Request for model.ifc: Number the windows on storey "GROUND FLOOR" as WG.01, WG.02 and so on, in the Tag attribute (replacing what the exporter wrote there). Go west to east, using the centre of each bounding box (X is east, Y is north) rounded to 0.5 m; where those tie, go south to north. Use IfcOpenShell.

First a look at what the model holds.

```python
import ifcopenshell
import ifcopenshell.util.element
import ifcopenshell.util.placement

model = ifcopenshell.open("model.ifc")
print(model.schema)
storey = next(s for s in model.by_type("IfcBuildingStorey") if s.Name == "GROUND FLOOR")
windows = [e for e in ifcopenshell.util.element.get_decomposition(storey) if e.is_a("IfcWindow")]
for e in sorted(windows, key=lambda e: e.id()):
    origin = ifcopenshell.util.placement.get_local_placement(e.ObjectPlacement)[:3, 3]
    print(e.id(), e.Tag, e.Name, origin.round(2) + 0.0, sep=" | ")
```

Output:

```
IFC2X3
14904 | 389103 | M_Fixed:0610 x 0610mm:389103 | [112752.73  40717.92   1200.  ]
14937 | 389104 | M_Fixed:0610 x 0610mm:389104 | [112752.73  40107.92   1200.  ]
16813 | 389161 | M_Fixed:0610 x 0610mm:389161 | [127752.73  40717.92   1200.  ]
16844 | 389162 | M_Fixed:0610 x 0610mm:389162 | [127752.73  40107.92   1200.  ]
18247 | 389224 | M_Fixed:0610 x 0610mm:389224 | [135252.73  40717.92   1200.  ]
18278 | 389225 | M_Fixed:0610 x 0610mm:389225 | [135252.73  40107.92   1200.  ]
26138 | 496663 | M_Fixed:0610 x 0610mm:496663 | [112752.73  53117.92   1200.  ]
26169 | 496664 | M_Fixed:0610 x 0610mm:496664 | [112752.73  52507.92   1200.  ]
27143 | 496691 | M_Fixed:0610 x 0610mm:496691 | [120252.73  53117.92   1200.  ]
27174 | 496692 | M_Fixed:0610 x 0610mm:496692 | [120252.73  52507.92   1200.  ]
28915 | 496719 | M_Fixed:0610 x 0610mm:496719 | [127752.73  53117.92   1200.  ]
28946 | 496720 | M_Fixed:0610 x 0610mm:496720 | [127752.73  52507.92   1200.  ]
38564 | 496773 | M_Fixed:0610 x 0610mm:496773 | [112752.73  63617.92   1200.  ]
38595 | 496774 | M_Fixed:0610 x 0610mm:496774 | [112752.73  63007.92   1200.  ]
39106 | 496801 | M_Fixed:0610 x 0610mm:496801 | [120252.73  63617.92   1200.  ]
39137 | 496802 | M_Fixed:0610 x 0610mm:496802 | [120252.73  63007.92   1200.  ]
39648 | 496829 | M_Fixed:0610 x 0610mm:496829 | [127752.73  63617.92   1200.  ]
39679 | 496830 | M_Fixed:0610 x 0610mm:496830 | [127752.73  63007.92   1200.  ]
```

```python
import ifcopenshell
import ifcopenshell.geom
import ifcopenshell.util.element
import ifcopenshell.util.shape

model = ifcopenshell.open("model.ifc")
settings = ifcopenshell.geom.settings()
settings.set("use-world-coords", True)


def centre(element):
    shape = ifcopenshell.geom.create_shape(settings, element)
    return ifcopenshell.util.shape.get_bbox_centroid(shape.geometry)


storey = next(s for s in model.by_type("IfcBuildingStorey") if s.Name == "GROUND FLOOR")
windows = [e for e in ifcopenshell.util.element.get_decomposition(storey) if e.is_a("IfcWindow")]

# Insertion points can sit at a corner or the storey origin, so sort by the geometry (in metres).
centres = {e: centre(e) for e in windows}
windows.sort(key=lambda e: (round(centres[e][0] / 0.5), centres[e][1]))

for i, e in enumerate(windows, start=1):
    number = f"WG.{i:02d}"
    e.Tag = number
    print(e.id(), number)

model.write("model_updated.ifc")
```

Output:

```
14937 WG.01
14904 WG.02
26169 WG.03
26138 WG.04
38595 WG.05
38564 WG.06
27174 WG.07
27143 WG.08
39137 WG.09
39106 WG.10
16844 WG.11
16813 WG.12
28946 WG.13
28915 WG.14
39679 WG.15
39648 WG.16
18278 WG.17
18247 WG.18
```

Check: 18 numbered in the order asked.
